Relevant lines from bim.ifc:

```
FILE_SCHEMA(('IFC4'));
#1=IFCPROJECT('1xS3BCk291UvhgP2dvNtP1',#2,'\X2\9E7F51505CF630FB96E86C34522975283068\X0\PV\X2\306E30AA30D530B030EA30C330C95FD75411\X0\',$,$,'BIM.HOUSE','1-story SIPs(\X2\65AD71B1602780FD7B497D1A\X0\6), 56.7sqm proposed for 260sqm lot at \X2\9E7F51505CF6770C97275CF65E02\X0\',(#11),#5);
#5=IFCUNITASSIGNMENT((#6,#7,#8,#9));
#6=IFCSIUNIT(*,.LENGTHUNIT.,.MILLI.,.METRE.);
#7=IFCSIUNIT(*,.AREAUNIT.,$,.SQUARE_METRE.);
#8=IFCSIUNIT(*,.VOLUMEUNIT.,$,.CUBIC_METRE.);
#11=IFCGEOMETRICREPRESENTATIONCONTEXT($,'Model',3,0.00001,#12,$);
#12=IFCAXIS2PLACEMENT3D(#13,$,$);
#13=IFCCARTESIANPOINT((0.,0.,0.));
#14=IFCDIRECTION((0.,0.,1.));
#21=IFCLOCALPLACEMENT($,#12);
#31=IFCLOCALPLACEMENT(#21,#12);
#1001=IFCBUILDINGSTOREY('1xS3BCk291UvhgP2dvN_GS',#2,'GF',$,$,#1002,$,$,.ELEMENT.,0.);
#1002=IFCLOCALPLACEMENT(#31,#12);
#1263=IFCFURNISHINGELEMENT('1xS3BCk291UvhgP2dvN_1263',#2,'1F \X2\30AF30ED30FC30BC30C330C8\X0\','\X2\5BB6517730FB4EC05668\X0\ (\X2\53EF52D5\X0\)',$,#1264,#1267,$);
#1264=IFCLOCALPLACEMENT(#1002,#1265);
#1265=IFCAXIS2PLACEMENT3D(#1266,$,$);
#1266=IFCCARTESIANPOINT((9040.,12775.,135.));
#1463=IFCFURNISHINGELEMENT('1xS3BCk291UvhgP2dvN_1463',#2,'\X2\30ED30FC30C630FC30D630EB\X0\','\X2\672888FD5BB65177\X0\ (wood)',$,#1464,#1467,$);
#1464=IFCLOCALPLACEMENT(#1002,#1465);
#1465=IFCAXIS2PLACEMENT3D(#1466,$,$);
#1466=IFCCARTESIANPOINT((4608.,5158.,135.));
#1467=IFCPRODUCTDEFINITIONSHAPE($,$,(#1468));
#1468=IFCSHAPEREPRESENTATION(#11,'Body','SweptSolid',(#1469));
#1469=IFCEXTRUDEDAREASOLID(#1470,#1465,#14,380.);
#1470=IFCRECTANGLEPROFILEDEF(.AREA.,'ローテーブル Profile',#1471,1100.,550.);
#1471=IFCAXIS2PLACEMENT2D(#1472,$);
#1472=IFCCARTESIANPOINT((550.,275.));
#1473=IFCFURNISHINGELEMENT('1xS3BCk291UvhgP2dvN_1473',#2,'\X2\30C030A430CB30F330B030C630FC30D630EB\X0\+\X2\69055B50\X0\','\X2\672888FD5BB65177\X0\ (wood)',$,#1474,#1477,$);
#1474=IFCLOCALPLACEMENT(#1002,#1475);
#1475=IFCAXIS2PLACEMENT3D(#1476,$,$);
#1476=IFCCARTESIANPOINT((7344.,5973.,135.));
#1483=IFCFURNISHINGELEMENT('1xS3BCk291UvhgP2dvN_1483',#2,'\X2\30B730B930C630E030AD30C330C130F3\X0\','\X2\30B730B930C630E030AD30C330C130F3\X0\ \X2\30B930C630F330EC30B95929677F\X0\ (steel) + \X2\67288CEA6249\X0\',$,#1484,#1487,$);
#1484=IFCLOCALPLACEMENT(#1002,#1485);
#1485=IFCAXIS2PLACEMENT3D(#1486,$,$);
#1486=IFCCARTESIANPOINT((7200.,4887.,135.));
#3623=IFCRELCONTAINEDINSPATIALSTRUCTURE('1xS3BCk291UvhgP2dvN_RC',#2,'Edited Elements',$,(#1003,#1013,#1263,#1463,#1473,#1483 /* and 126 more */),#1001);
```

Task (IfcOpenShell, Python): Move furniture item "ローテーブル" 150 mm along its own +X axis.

```python
import ifcopenshell
import ifcopenshell.api.geometry
import ifcopenshell.util.placement

model = ifcopenshell.open("bim.ifc")

item = model.by_guid("1xS3BCk291UvhgP2dvN_1463")
matrix = ifcopenshell.util.placement.get_local_placement(item.ObjectPlacement)
matrix[:3, 3] += matrix[:3, 0] * 150.0
ifcopenshell.api.geometry.edit_object_placement(model, product=item, matrix=matrix, is_si=False)

print(ifcopenshell.util.placement.get_local_placement(item.ObjectPlacement).round(3) + 0.0)

model.write("bim_v2.ifc")
```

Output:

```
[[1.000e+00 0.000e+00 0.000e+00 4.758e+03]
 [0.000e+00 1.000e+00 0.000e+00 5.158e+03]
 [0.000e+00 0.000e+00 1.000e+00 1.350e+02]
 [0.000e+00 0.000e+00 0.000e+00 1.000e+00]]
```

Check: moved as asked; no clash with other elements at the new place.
